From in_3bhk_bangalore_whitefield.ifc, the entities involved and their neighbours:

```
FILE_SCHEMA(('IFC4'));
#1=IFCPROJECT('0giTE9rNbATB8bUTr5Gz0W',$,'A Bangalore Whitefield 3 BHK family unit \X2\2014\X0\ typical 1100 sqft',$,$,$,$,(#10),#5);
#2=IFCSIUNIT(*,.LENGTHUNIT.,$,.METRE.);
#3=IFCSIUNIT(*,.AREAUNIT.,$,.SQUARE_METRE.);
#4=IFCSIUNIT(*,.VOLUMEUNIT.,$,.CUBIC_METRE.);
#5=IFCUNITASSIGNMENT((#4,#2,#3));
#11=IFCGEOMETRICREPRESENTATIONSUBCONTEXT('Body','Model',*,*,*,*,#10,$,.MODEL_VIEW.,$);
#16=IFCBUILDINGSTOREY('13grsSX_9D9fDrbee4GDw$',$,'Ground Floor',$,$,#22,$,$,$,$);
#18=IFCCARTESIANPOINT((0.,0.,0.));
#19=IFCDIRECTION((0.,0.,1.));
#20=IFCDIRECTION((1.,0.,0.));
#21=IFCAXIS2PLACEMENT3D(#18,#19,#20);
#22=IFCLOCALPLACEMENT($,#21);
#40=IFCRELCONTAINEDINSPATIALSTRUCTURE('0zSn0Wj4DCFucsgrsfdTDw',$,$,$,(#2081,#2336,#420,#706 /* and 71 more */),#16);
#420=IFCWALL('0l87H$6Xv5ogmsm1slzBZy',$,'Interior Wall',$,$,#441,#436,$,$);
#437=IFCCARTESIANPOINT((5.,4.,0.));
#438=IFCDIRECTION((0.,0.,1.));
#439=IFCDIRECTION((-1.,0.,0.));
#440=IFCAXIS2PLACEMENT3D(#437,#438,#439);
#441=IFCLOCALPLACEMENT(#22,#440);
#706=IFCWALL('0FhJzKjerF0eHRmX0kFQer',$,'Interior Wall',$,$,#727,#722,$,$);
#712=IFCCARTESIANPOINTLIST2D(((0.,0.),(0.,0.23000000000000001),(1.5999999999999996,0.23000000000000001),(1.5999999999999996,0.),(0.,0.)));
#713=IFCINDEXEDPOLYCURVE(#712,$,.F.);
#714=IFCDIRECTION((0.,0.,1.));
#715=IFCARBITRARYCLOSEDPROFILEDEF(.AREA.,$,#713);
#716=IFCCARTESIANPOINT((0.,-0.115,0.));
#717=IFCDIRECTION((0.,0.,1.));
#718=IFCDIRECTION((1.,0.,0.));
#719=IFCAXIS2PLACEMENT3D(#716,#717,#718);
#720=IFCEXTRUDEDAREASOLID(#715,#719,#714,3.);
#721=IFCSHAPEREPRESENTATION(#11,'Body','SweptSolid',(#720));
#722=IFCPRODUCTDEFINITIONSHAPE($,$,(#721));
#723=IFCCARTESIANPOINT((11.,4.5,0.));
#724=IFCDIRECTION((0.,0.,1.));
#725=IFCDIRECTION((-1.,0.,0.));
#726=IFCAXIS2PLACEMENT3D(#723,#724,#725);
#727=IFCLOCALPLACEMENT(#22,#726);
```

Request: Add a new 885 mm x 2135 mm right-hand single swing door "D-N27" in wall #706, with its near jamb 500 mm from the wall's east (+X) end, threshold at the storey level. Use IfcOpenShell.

```python
import numpy as np
import ifcopenshell
import ifcopenshell.api.feature
import ifcopenshell.api.geometry
import ifcopenshell.api.root
import ifcopenshell.api.spatial
import ifcopenshell.geom
import ifcopenshell.util.element
import ifcopenshell.util.placement
import ifcopenshell.util.representation
import ifcopenshell.util.shape
import ifcopenshell.util.unit

model = ifcopenshell.open("in_3bhk_bangalore_whitefield.ifc")
unit_scale = ifcopenshell.util.unit.calculate_unit_scale(model)
settings = ifcopenshell.geom.settings()


def volume(element):
    """Net volume in cubic metres, openings subtracted."""
    shape = ifcopenshell.geom.create_shape(settings, element)
    return ifcopenshell.util.shape.get_volume(shape.geometry)


wall = model.by_guid("0FhJzKjerF0eHRmX0kFQer")
storey = ifcopenshell.util.element.get_container(wall, ifc_class="IfcBuildingStorey")
context = ifcopenshell.util.representation.get_context(model, "Model", "Body", "MODEL_VIEW")
before = volume(wall)

width, height, from_end, sill = 0.885, 2.135, 0.5, 0.0  # metres

# The wall runs along its own X axis, and the end named is its -X end.
wall_shape = ifcopenshell.geom.create_shape(settings, wall)
x, y, z = ifcopenshell.util.shape.get_vertices(wall_shape.geometry).T
start = x.min() + from_end
face, thickness = float(y.min()), float(y.max() - y.min())
wall_matrix = ifcopenshell.util.placement.get_local_placement(wall.ObjectPlacement)
level = ifcopenshell.util.placement.get_local_placement(storey.ObjectPlacement)[2, 3]


def in_wall(x, y):
    """Placement at x, y metres in the wall's axes, at sill height."""
    matrix = wall_matrix.copy()
    matrix[:, 3] = wall_matrix @ np.array([x / unit_scale, y / unit_scale, 0.0, 1.0])
    matrix[2, 3] = level + sill / unit_scale
    return matrix


# Opening: a box that overshoots both wall faces by 50 mm.
opening = ifcopenshell.api.root.create_entity(model, ifc_class="IfcOpeningElement", predefined_type="OPENING")
box = ifcopenshell.api.geometry.add_wall_representation(
    model, context=context, length=width, height=height, thickness=thickness + 0.1
)
ifcopenshell.api.geometry.assign_representation(model, product=opening, representation=box)
ifcopenshell.api.geometry.edit_object_placement(model, product=opening, matrix=in_wall(start, face - 0.05), is_si=False)
ifcopenshell.api.feature.add_feature(model, feature=opening, element=wall)

door = ifcopenshell.api.root.create_entity(model, ifc_class="IfcDoor", name="D-N27", predefined_type="DOOR")
door.OverallWidth, door.OverallHeight = width / unit_scale, height / unit_scale
door.OperationType = "SINGLE_SWING_RIGHT"
body = ifcopenshell.api.geometry.add_door_representation(
    model,
    context=context,
    overall_width=door.OverallWidth,
    overall_height=door.OverallHeight,
    operation_type="SINGLE_SWING_RIGHT",
    lining_properties={"LiningDepth": thickness / unit_scale, "ThresholdDepth": thickness / unit_scale},
)
ifcopenshell.api.geometry.assign_representation(model, product=door, representation=body)
ifcopenshell.api.spatial.assign_container(model, products=[door], relating_structure=storey)
ifcopenshell.api.feature.add_filling(model, opening=opening, element=door)

# The lining spans the wall, so the door starts at the wall face.
ifcopenshell.api.geometry.edit_object_placement(model, product=door, matrix=in_wall(start, face), is_si=False)

after = volume(wall)

print(f"wall volume {before:.3f} -> {after:.3f} m3")

model.write("in_3bhk_bangalore_whitefield_v2.ifc")
```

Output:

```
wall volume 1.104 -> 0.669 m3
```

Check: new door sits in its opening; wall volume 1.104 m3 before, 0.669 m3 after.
